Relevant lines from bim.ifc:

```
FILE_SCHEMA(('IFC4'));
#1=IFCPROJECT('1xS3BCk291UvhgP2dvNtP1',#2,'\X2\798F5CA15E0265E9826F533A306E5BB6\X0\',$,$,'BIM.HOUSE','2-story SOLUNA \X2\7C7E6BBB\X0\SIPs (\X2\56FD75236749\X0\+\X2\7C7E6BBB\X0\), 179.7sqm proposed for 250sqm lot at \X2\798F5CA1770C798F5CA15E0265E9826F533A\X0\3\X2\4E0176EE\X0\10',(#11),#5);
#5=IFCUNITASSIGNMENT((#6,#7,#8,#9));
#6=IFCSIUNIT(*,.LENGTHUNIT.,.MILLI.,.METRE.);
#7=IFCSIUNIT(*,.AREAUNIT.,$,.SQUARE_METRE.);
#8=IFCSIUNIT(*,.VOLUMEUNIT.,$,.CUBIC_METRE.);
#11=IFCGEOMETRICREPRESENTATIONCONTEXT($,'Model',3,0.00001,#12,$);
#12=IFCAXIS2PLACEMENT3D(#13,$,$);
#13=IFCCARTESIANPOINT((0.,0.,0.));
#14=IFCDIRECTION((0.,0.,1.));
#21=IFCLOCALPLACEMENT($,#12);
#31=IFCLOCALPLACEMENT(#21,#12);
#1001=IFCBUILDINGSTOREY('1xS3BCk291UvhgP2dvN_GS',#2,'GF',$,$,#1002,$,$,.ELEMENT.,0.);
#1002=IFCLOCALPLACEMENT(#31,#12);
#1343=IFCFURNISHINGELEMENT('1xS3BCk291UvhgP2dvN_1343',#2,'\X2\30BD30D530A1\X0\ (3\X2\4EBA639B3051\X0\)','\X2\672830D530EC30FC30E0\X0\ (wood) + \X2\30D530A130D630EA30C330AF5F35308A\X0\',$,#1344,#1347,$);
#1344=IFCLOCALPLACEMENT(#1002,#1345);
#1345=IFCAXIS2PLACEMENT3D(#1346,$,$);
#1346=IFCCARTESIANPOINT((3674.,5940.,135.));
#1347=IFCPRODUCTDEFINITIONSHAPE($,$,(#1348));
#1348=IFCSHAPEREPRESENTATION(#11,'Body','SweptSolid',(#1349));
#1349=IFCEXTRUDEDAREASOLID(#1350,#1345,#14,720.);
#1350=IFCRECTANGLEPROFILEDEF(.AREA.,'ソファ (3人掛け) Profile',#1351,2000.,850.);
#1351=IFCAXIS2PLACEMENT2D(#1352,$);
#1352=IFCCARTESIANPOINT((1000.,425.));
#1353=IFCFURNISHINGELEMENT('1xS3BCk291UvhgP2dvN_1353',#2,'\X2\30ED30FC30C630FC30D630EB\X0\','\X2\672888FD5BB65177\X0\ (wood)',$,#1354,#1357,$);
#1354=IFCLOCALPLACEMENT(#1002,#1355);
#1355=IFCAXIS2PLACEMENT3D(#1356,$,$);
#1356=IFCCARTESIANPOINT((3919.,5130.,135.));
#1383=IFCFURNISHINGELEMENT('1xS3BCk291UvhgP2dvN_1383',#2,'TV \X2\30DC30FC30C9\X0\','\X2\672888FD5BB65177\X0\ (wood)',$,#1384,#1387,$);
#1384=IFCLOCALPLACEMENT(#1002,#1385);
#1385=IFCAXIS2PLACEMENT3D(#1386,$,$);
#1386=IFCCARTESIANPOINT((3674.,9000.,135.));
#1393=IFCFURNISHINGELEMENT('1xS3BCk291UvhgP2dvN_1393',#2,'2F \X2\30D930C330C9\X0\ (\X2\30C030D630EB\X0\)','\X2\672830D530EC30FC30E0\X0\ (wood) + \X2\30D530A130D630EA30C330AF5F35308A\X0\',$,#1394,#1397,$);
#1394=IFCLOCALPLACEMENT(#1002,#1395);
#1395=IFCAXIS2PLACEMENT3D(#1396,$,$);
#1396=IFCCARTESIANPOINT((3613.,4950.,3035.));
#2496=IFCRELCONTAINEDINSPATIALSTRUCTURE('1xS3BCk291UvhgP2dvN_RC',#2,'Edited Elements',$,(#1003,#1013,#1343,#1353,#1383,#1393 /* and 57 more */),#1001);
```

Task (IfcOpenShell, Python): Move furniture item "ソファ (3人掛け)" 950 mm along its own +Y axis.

```python
import ifcopenshell
import ifcopenshell.api.geometry
import ifcopenshell.util.placement
import ifcopenshell.util.unit

model = ifcopenshell.open("bim.ifc")
unit_scale = ifcopenshell.util.unit.calculate_unit_scale(model)

item = model.by_id(1343)
matrix = ifcopenshell.util.placement.get_local_placement(item.ObjectPlacement)
matrix[:3, 3] += matrix[:3, 1] * 0.95 / unit_scale
ifcopenshell.api.geometry.edit_object_placement(model, product=item, matrix=matrix, is_si=False)

print(ifcopenshell.util.placement.get_local_placement(item.ObjectPlacement).round(3) + 0.0)

model.write("bim_rev.ifc")
```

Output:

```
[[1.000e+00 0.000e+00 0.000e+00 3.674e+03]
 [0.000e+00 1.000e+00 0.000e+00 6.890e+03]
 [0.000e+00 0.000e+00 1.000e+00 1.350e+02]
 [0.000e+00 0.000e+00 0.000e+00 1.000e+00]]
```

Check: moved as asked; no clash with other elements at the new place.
